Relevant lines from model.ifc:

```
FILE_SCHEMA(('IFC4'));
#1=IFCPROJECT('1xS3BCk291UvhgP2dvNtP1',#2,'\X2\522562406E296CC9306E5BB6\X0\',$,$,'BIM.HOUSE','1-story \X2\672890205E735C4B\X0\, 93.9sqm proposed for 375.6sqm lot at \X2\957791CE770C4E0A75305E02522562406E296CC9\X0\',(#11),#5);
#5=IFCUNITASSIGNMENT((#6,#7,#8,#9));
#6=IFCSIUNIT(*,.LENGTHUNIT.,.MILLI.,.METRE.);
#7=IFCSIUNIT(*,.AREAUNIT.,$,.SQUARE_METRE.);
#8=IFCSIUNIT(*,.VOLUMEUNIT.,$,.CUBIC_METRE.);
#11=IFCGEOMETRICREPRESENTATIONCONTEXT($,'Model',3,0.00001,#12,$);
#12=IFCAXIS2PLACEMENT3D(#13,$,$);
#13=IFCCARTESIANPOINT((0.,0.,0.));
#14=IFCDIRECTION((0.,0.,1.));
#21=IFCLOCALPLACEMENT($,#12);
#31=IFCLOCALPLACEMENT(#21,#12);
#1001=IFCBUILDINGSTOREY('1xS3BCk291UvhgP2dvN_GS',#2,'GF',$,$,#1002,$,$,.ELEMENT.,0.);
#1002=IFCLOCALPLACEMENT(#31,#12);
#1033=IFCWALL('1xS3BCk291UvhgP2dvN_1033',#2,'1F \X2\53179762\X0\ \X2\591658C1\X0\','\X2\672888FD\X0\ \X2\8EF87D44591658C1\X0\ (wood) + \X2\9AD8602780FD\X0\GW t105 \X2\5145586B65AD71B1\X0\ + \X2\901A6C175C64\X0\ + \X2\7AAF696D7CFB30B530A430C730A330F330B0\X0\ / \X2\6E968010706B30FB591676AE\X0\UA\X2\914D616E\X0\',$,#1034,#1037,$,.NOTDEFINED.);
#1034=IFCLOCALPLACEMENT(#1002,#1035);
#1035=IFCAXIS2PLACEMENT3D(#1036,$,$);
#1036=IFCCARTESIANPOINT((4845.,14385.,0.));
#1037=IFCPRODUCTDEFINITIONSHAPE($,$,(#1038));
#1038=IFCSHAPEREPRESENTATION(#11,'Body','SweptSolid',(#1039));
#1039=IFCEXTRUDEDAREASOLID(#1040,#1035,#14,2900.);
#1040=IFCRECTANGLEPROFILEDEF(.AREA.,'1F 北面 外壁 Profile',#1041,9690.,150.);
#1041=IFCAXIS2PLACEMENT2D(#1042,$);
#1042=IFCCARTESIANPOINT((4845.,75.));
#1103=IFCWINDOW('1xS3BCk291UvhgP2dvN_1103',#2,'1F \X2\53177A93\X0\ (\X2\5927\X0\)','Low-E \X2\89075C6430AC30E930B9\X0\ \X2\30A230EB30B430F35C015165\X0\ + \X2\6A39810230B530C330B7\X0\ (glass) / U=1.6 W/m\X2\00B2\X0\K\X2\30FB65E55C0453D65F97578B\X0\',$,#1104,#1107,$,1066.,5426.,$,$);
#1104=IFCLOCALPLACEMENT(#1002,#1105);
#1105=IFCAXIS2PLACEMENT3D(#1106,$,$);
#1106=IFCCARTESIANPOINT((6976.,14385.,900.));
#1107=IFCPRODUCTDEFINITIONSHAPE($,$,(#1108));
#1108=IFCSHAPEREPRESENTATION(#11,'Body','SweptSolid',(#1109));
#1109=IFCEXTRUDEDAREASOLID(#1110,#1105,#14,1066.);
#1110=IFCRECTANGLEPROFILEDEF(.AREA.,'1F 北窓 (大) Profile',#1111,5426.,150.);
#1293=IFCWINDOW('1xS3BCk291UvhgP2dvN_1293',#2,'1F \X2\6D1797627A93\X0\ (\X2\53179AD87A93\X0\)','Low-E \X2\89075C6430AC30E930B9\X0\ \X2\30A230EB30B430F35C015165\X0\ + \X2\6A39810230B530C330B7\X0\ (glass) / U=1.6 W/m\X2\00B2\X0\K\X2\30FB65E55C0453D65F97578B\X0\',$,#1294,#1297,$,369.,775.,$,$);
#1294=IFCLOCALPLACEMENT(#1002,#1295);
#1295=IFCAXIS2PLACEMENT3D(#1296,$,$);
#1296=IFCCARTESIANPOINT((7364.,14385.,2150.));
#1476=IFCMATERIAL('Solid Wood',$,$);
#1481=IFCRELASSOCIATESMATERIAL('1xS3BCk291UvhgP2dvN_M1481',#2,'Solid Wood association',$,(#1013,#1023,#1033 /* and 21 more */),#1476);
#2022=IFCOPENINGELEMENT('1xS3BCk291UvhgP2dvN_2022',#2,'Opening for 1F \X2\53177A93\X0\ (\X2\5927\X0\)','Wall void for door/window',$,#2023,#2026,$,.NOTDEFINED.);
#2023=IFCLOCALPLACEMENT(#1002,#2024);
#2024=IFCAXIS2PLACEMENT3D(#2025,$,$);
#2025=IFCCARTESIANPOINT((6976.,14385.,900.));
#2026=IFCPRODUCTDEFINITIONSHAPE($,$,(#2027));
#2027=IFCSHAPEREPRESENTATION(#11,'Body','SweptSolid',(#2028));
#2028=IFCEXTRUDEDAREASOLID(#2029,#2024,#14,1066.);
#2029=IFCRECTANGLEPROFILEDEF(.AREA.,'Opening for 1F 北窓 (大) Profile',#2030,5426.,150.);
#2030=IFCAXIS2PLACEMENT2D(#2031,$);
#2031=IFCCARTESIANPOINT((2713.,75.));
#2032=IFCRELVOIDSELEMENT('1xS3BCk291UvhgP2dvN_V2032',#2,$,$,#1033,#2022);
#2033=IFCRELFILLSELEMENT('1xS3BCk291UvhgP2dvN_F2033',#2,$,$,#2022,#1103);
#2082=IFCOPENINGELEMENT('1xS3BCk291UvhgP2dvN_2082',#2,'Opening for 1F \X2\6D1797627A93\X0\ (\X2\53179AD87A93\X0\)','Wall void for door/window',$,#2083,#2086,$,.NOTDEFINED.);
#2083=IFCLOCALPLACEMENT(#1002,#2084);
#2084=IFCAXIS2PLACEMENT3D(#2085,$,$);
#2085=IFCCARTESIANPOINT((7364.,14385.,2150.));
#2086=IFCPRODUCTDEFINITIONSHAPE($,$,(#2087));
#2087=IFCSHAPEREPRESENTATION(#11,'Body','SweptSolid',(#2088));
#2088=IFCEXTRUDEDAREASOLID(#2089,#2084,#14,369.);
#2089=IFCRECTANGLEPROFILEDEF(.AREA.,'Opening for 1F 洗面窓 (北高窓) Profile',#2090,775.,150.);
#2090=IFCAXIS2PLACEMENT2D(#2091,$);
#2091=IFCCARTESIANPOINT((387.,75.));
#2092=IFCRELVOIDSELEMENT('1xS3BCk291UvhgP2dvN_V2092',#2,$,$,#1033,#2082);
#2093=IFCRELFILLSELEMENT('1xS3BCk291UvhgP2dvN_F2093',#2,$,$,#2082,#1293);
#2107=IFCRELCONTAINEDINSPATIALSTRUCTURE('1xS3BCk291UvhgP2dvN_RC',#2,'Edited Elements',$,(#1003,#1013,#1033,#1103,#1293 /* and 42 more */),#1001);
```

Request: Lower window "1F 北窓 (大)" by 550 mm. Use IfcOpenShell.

```python
import numpy as np
import ifcopenshell
import ifcopenshell.api.geometry
import ifcopenshell.util.placement
import ifcopenshell.util.unit

model = ifcopenshell.open("model.ifc")
unit_scale = ifcopenshell.util.unit.calculate_unit_scale(model)

window = model.by_id(1103)
opening = window.FillsVoids[0].RelatingOpeningElement
dz = -550.0

shift = np.array([0.0, 0.0, dz])
# The window is not placed relative to its opening, so move both.
for product in (opening, window):
    matrix = ifcopenshell.util.placement.get_local_placement(product.ObjectPlacement)
    matrix[:3, 3] += shift
    ifcopenshell.api.geometry.edit_object_placement(model, product=product, matrix=matrix, is_si=False)

print(f"moved by {dz * unit_scale:+.3f} m")

model.write("model_edited.ifc")
```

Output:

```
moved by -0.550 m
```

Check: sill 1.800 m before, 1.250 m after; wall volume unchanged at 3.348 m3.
